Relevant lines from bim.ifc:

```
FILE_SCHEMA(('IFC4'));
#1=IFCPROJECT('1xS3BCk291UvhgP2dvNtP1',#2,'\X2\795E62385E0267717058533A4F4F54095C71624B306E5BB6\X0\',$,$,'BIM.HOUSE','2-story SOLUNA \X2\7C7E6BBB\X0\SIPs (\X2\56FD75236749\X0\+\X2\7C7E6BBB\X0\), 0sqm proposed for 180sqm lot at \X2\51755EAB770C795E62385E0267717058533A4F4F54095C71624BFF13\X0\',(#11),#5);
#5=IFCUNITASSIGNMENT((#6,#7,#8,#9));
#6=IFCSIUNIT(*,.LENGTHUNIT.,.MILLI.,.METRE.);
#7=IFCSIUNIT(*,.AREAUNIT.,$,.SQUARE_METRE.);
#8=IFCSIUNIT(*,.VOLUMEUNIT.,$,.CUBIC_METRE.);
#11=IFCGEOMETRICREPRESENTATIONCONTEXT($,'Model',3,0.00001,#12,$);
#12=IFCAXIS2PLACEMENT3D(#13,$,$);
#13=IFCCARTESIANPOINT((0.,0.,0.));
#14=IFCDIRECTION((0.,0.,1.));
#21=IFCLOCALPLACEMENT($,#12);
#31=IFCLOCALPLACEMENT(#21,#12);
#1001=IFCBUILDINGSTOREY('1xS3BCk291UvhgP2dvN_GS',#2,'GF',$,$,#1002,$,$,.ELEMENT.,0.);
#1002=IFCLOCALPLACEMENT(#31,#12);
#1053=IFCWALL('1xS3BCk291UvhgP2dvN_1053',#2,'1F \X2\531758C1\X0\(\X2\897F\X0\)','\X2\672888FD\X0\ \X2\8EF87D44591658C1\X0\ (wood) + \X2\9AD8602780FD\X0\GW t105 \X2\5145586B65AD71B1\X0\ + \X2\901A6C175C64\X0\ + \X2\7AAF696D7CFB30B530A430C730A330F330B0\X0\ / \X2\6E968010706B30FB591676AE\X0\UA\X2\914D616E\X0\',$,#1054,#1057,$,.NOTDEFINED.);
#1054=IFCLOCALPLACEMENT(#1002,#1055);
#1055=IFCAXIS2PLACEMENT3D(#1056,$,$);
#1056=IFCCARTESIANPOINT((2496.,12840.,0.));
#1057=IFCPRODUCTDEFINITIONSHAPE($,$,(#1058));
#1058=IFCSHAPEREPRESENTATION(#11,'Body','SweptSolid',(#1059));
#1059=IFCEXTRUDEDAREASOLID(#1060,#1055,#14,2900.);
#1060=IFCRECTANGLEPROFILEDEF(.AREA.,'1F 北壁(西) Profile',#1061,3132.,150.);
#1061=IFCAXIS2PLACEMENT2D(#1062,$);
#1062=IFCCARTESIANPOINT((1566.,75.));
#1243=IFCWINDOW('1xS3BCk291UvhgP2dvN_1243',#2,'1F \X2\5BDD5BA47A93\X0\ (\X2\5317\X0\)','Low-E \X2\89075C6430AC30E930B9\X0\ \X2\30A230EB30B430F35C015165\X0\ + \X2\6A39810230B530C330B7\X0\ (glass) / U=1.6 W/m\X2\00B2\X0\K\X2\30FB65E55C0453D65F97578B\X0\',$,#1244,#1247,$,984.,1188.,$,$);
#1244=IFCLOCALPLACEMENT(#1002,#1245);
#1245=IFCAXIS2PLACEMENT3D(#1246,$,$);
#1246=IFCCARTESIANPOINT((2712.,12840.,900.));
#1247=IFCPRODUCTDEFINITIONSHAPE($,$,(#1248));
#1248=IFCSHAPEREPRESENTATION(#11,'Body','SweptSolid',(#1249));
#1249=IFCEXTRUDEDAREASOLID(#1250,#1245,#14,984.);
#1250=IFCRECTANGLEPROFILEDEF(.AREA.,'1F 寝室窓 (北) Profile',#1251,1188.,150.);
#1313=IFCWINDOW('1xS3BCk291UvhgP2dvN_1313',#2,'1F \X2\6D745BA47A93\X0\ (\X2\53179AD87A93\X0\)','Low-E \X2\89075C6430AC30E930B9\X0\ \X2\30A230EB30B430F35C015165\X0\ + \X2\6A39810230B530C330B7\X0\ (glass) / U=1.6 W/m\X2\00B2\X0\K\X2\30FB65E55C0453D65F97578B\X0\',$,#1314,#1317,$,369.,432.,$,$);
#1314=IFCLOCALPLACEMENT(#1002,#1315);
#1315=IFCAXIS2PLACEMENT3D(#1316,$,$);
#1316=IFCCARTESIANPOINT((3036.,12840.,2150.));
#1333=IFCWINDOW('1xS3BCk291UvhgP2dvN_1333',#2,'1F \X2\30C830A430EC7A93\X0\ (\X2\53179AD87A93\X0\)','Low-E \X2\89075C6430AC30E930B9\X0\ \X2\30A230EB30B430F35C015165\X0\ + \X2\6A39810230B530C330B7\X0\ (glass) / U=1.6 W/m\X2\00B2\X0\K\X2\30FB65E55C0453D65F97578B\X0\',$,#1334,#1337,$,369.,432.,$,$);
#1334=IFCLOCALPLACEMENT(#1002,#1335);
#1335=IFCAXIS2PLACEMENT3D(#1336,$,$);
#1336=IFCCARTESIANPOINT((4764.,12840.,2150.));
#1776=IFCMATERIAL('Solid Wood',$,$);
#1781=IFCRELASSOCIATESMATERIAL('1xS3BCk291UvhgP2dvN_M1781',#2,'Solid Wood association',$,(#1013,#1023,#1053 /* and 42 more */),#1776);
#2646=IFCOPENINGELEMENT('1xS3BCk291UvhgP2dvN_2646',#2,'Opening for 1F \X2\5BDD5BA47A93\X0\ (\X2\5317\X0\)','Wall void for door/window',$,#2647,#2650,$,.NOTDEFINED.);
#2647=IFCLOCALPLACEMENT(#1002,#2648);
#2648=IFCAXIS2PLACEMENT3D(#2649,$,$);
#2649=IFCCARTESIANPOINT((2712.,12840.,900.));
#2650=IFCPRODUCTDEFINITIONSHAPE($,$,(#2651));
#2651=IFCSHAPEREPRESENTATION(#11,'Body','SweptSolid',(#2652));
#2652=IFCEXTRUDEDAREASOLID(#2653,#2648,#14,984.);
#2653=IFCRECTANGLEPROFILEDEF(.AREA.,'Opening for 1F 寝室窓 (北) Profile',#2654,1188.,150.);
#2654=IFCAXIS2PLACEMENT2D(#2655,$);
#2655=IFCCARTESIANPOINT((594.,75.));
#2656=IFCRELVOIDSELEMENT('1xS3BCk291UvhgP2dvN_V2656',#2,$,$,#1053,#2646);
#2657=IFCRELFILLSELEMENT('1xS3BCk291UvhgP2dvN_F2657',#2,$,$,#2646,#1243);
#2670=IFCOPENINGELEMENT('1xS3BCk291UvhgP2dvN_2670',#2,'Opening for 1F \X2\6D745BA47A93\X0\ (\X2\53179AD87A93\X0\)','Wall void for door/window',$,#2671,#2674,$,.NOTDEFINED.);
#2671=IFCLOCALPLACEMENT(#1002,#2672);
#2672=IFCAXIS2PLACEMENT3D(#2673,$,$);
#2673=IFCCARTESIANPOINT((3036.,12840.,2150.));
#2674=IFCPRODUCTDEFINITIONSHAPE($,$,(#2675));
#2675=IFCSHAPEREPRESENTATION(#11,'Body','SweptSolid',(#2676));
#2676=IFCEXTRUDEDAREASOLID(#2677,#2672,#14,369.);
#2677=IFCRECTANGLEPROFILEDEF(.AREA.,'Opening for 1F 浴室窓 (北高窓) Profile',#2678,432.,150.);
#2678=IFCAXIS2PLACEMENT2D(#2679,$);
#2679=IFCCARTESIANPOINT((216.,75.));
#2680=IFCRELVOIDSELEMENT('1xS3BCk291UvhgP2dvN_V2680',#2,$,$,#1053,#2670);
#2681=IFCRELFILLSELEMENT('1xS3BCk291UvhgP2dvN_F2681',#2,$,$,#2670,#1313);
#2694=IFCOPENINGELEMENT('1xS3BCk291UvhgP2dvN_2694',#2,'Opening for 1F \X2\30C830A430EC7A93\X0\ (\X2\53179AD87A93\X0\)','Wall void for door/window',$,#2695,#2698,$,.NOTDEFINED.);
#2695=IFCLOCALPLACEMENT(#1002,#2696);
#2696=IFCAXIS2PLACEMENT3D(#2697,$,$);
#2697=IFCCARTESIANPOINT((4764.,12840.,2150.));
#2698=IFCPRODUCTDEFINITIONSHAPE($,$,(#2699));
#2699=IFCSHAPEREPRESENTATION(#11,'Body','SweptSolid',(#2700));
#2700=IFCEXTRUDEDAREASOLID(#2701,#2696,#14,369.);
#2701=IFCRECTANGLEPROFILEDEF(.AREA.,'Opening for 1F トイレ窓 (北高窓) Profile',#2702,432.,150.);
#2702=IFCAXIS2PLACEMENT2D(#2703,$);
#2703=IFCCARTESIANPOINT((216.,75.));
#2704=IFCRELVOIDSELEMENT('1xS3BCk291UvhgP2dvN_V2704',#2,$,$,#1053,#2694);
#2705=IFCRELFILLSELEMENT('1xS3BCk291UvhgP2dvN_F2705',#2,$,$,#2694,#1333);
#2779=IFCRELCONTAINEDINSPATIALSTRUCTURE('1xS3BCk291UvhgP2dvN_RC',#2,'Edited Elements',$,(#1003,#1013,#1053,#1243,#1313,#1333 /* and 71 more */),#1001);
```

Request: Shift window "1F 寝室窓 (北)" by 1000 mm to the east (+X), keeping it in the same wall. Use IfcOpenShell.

```python
import ifcopenshell
import ifcopenshell.api.geometry
import ifcopenshell.util.placement
import ifcopenshell.util.unit

model = ifcopenshell.open("bim.ifc")
unit_scale = ifcopenshell.util.unit.calculate_unit_scale(model)

window = model.by_guid("1xS3BCk291UvhgP2dvN_1243")
opening = window.FillsVoids[0].RelatingOpeningElement
wall = opening.VoidsElements[0].RelatingBuildingElement

wall_matrix = ifcopenshell.util.placement.get_local_placement(wall.ObjectPlacement)
shift = wall_matrix[:3, 0] * 1 / unit_scale
before = ifcopenshell.util.placement.get_local_placement(window.ObjectPlacement)[:3, 3].copy()

# The window is not placed relative to its opening, so move both.
for product in (opening, window):
    matrix = ifcopenshell.util.placement.get_local_placement(product.ObjectPlacement)
    matrix[:3, 3] += shift
    ifcopenshell.api.geometry.edit_object_placement(model, product=product, matrix=matrix, is_si=False)

after = ifcopenshell.util.placement.get_local_placement(window.ObjectPlacement)[:3, 3]
print("window moved by", (after - before).round(3) + 0.0)

model.write("bim_rev.ifc")
```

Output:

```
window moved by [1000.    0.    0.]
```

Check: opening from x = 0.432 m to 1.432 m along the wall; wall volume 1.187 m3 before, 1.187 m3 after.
